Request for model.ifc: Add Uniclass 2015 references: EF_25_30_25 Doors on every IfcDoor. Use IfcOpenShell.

First a look at what the model holds.

```python
import ifcopenshell

model = ifcopenshell.open("model.ifc")
print(model.schema)
print("classifications:", [c.Name for c in model.by_type("IfcClassification")])
for ifc_class in ("IfcDoor", "IfcRoof", "IfcStair", "IfcWall", "IfcWindow"):
    print(ifc_class, len(model.by_type(ifc_class)))
```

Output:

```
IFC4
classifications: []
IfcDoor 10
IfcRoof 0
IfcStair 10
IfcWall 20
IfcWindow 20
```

```python
import ifcopenshell
import ifcopenshell.api.classification

model = ifcopenshell.open("model.ifc")

system = ifcopenshell.api.classification.add_classification(model, classification="Uniclass 2015")

codes = {
    "IfcDoor": ("EF_25_30_25", "Doors"),
}
for ifc_class, (code, name) in codes.items():
    products = model.by_type(ifc_class)
    ifcopenshell.api.classification.add_reference(
        model, products=products, classification=system, identification=code, name=name
    )
    print(code, len(products))

model.write("model_rev.ifc")
```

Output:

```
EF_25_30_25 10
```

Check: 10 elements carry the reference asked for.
